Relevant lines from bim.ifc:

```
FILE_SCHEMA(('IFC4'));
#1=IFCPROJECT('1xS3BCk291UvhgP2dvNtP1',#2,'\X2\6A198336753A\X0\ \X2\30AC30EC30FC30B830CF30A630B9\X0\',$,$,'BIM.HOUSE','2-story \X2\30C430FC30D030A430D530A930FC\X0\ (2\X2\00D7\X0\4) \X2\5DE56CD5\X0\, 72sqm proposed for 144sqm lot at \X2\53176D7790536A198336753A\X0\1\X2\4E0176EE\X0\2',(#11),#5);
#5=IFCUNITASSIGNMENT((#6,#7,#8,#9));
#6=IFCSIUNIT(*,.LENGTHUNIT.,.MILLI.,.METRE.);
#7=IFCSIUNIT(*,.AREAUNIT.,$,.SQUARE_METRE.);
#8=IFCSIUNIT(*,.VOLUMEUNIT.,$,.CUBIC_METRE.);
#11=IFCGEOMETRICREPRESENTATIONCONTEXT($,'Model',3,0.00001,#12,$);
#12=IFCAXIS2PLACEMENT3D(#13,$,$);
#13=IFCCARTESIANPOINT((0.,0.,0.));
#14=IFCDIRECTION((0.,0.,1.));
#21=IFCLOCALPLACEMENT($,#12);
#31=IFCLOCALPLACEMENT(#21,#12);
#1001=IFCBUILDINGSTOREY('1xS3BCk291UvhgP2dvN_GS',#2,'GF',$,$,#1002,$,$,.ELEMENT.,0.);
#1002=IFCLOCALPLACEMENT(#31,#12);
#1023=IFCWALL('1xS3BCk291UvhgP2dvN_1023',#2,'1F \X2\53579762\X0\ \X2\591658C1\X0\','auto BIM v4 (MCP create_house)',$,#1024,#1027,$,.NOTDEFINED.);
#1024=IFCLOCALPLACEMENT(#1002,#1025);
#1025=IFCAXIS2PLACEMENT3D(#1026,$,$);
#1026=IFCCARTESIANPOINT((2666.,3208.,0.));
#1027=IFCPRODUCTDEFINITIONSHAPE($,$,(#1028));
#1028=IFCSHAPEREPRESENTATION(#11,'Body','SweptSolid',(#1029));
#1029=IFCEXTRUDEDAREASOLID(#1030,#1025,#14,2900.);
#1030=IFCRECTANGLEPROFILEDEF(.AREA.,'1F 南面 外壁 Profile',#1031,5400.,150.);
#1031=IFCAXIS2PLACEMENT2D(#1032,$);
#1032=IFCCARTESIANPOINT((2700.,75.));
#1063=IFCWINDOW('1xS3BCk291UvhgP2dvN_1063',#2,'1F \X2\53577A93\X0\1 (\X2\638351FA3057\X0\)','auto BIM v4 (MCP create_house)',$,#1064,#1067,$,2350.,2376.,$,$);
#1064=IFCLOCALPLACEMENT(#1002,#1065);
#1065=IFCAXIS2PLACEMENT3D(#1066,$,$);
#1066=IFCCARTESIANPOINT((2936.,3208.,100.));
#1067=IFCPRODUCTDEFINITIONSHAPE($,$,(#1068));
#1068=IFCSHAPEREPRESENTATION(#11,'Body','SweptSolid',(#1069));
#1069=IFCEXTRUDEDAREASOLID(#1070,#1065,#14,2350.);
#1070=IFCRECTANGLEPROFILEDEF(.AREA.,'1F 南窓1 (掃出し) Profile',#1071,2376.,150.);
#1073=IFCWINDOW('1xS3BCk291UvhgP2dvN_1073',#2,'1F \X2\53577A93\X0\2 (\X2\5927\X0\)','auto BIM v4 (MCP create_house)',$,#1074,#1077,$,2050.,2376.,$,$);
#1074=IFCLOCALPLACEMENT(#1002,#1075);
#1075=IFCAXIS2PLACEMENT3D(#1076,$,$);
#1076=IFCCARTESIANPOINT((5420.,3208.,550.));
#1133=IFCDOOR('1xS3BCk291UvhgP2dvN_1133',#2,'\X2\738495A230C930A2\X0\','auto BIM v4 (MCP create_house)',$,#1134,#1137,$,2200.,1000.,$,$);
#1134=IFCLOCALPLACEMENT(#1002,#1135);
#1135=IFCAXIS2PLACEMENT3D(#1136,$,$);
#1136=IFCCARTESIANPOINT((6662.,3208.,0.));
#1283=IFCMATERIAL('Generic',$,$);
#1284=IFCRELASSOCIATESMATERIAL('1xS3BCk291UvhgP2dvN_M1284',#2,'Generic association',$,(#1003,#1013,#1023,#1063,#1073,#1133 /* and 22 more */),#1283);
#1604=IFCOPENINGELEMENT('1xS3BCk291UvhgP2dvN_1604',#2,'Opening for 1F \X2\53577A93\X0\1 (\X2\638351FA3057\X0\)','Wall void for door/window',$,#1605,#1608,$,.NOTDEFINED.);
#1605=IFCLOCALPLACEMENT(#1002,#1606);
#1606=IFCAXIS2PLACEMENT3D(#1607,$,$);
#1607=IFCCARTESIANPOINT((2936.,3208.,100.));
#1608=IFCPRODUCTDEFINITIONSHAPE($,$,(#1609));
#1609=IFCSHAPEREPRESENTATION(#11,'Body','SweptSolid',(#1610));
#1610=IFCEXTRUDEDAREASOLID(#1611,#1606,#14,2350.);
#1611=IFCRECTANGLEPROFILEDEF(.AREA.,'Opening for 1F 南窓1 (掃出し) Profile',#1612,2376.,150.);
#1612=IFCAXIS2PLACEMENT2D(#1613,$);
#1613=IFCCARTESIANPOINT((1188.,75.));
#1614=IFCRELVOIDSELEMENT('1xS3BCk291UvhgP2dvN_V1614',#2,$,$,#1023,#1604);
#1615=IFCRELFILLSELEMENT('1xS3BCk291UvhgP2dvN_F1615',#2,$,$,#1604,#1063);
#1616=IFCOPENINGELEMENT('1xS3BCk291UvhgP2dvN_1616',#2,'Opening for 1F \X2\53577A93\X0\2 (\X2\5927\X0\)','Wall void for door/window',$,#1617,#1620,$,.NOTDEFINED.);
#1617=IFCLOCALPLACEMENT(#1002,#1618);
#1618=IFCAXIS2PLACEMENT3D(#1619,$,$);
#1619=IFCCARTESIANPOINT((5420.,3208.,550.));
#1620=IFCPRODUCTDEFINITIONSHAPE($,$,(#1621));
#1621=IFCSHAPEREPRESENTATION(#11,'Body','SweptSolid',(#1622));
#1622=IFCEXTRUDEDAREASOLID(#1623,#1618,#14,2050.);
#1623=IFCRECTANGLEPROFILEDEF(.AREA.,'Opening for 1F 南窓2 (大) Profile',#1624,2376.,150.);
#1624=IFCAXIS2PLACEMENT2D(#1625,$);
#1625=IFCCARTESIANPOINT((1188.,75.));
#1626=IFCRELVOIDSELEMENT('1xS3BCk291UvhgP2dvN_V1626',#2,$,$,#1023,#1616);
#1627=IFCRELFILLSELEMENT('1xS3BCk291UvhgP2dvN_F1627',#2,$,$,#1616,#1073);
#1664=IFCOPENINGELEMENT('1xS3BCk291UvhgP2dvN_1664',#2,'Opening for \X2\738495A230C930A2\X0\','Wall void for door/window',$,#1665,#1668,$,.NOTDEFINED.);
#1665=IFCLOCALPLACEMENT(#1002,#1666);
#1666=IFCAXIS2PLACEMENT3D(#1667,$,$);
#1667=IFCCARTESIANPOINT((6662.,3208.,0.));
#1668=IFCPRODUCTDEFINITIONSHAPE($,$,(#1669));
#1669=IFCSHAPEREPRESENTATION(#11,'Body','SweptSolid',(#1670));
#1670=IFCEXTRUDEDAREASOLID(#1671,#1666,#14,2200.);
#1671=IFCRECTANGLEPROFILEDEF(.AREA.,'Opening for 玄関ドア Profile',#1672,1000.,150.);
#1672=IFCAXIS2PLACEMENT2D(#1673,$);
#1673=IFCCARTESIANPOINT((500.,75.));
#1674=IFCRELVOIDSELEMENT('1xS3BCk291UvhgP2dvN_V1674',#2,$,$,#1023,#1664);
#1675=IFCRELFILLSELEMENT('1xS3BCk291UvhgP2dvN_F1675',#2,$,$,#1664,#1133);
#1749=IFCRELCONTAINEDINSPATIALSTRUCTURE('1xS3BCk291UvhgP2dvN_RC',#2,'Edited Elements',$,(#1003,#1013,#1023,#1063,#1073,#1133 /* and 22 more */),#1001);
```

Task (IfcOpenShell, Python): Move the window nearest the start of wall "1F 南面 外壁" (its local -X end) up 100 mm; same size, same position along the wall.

```python
import numpy as np
import ifcopenshell
import ifcopenshell.api.geometry
import ifcopenshell.util.placement
import ifcopenshell.util.unit

model = ifcopenshell.open("bim.ifc")
unit_scale = ifcopenshell.util.unit.calculate_unit_scale(model)

window = model.by_guid("1xS3BCk291UvhgP2dvN_1063")
opening = window.FillsVoids[0].RelatingOpeningElement
dz = 100.0

shift = np.array([0.0, 0.0, dz])
# The window is not placed relative to its opening, so move both.
for product in (opening, window):
    matrix = ifcopenshell.util.placement.get_local_placement(product.ObjectPlacement)
    matrix[:3, 3] += shift
    ifcopenshell.api.geometry.edit_object_placement(model, product=product, matrix=matrix, is_si=False)

print(f"moved by {dz * unit_scale:+.3f} m")

model.write("bim_updated.ifc")
```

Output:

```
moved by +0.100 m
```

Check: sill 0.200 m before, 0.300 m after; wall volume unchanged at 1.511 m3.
